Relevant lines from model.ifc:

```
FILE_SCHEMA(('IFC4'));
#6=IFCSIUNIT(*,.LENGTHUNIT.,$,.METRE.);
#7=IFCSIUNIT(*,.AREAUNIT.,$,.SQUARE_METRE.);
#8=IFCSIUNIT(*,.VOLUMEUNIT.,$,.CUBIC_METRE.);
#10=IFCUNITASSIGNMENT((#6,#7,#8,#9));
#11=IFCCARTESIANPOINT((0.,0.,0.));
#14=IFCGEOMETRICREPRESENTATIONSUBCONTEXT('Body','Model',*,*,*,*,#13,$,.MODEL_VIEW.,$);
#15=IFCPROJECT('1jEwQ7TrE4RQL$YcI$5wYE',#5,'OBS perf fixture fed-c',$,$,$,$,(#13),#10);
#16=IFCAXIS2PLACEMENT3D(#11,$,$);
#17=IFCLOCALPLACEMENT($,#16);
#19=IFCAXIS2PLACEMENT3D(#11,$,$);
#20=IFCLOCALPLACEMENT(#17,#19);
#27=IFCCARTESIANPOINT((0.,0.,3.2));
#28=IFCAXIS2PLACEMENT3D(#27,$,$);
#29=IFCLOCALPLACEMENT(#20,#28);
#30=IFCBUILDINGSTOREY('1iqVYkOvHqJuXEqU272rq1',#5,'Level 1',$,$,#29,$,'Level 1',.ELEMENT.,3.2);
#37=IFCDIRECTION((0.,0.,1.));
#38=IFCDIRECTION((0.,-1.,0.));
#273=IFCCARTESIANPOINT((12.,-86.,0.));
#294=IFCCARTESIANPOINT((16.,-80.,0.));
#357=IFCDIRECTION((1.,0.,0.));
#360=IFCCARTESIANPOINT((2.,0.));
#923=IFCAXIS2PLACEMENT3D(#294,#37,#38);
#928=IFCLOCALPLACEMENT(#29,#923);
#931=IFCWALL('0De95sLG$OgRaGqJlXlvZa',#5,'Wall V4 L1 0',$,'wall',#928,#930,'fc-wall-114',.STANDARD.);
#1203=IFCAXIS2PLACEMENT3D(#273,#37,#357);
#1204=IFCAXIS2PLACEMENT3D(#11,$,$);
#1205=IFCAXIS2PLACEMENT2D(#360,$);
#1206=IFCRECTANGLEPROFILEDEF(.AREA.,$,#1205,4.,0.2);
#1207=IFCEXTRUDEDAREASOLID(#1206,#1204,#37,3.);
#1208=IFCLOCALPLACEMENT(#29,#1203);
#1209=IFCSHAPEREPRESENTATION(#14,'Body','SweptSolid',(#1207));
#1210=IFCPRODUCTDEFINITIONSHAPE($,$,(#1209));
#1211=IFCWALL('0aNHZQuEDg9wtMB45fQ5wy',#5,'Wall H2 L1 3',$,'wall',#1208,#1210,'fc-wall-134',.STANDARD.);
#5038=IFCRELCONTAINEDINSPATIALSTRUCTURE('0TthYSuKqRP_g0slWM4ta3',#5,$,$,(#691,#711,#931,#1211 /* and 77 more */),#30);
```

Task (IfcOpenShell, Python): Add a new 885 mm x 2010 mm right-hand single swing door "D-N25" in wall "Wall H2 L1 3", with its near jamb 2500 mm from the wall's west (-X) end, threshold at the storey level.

```python
import numpy as np
import ifcopenshell
import ifcopenshell.api.feature
import ifcopenshell.api.geometry
import ifcopenshell.api.root
import ifcopenshell.api.spatial
import ifcopenshell.geom
import ifcopenshell.util.element
import ifcopenshell.util.placement
import ifcopenshell.util.representation
import ifcopenshell.util.shape
import ifcopenshell.util.unit

model = ifcopenshell.open("model.ifc")
unit_scale = ifcopenshell.util.unit.calculate_unit_scale(model)
settings = ifcopenshell.geom.settings()


def volume(element):
    """Net volume in cubic metres, openings subtracted."""
    shape = ifcopenshell.geom.create_shape(settings, element)
    return ifcopenshell.util.shape.get_volume(shape.geometry)


wall = model.by_id(1211)
storey = ifcopenshell.util.element.get_container(wall, ifc_class="IfcBuildingStorey")
context = ifcopenshell.util.representation.get_context(model, "Model", "Body", "MODEL_VIEW")
before = volume(wall)

width, height, from_end, sill = 0.885, 2.01, 2.5, 0.0  # metres

# The wall runs along its own X axis, and the end named is its -X end.
wall_shape = ifcopenshell.geom.create_shape(settings, wall)
x, y, z = ifcopenshell.util.shape.get_vertices(wall_shape.geometry).T
start = x.min() + from_end
face, thickness = float(y.min()), float(y.max() - y.min())
wall_matrix = ifcopenshell.util.placement.get_local_placement(wall.ObjectPlacement)
level = ifcopenshell.util.placement.get_local_placement(storey.ObjectPlacement)[2, 3]


def in_wall(x, y):
    """Placement at x, y metres in the wall's axes, at sill height."""
    matrix = wall_matrix.copy()
    matrix[:, 3] = wall_matrix @ np.array([x / unit_scale, y / unit_scale, 0.0, 1.0])
    matrix[2, 3] = level + sill / unit_scale
    return matrix


# Opening: a box that overshoots both wall faces by 50 mm.
opening = ifcopenshell.api.root.create_entity(model, ifc_class="IfcOpeningElement", predefined_type="OPENING")
box = ifcopenshell.api.geometry.add_wall_representation(
    model, context=context, length=width, height=height, thickness=thickness + 0.1
)
ifcopenshell.api.geometry.assign_representation(model, product=opening, representation=box)
ifcopenshell.api.geometry.edit_object_placement(model, product=opening, matrix=in_wall(start, face - 0.05), is_si=False)
ifcopenshell.api.feature.add_feature(model, feature=opening, element=wall)

door = ifcopenshell.api.root.create_entity(model, ifc_class="IfcDoor", name="D-N25", predefined_type="DOOR")
door.OverallWidth, door.OverallHeight = width / unit_scale, height / unit_scale
door.OperationType = "SINGLE_SWING_RIGHT"
body = ifcopenshell.api.geometry.add_door_representation(
    model,
    context=context,
    overall_width=door.OverallWidth,
    overall_height=door.OverallHeight,
    operation_type="SINGLE_SWING_RIGHT",
    lining_properties={"LiningDepth": thickness / unit_scale, "ThresholdDepth": thickness / unit_scale},
)
ifcopenshell.api.geometry.assign_representation(model, product=door, representation=body)
ifcopenshell.api.spatial.assign_container(model, products=[door], relating_structure=storey)
ifcopenshell.api.feature.add_filling(model, opening=opening, element=door)

# The lining spans the wall, so the door starts at the wall face.
ifcopenshell.api.geometry.edit_object_placement(model, product=door, matrix=in_wall(start, face), is_si=False)

after = volume(wall)

print(f"wall volume {before:.3f} -> {after:.3f} m3")

model.write("model_v2.ifc")
```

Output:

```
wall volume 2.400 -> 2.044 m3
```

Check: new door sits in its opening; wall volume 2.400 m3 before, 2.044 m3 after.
